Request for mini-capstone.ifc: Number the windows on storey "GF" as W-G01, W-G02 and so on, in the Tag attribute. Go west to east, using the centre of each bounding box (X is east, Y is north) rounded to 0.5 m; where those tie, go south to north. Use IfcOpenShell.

First a look at what the model holds.

```python
import ifcopenshell
import ifcopenshell.util.element
import ifcopenshell.util.placement

model = ifcopenshell.open("mini-capstone.ifc")
print(model.schema)
storey = next(s for s in model.by_type("IfcBuildingStorey") if s.Name == "GF")
windows = [e for e in ifcopenshell.util.element.get_decomposition(storey) if e.is_a("IfcWindow")]
for e in sorted(windows, key=lambda e: e.id()):
    origin = ifcopenshell.util.placement.get_local_placement(e.ObjectPlacement)[:3, 3]
    print(e.id(), e.Tag, e.Name, origin.round(2) + 0.0, sep=" | ")
```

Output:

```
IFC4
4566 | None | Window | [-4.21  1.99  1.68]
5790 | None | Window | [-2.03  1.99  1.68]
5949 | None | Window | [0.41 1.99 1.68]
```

```python
import ifcopenshell
import ifcopenshell.geom
import ifcopenshell.util.element
import ifcopenshell.util.shape

model = ifcopenshell.open("mini-capstone.ifc")
settings = ifcopenshell.geom.settings()
settings.set("use-world-coords", True)


def centre(element):
    shape = ifcopenshell.geom.create_shape(settings, element)
    return ifcopenshell.util.shape.get_bbox_centroid(shape.geometry)


storey = next(s for s in model.by_type("IfcBuildingStorey") if s.Name == "GF")
windows = [e for e in ifcopenshell.util.element.get_decomposition(storey) if e.is_a("IfcWindow")]

# Insertion points can sit at a corner or the storey origin, so sort by the geometry (in metres).
centres = {e: centre(e) for e in windows}
windows.sort(key=lambda e: (round(centres[e][0] / 0.5), centres[e][1]))

for i, e in enumerate(windows, start=1):
    number = f"W-G{i:02d}"
    e.Tag = number
    print(e.id(), number)

model.write("mini-capstone_v2.ifc")
```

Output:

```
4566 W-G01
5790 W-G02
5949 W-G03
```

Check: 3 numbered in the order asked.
